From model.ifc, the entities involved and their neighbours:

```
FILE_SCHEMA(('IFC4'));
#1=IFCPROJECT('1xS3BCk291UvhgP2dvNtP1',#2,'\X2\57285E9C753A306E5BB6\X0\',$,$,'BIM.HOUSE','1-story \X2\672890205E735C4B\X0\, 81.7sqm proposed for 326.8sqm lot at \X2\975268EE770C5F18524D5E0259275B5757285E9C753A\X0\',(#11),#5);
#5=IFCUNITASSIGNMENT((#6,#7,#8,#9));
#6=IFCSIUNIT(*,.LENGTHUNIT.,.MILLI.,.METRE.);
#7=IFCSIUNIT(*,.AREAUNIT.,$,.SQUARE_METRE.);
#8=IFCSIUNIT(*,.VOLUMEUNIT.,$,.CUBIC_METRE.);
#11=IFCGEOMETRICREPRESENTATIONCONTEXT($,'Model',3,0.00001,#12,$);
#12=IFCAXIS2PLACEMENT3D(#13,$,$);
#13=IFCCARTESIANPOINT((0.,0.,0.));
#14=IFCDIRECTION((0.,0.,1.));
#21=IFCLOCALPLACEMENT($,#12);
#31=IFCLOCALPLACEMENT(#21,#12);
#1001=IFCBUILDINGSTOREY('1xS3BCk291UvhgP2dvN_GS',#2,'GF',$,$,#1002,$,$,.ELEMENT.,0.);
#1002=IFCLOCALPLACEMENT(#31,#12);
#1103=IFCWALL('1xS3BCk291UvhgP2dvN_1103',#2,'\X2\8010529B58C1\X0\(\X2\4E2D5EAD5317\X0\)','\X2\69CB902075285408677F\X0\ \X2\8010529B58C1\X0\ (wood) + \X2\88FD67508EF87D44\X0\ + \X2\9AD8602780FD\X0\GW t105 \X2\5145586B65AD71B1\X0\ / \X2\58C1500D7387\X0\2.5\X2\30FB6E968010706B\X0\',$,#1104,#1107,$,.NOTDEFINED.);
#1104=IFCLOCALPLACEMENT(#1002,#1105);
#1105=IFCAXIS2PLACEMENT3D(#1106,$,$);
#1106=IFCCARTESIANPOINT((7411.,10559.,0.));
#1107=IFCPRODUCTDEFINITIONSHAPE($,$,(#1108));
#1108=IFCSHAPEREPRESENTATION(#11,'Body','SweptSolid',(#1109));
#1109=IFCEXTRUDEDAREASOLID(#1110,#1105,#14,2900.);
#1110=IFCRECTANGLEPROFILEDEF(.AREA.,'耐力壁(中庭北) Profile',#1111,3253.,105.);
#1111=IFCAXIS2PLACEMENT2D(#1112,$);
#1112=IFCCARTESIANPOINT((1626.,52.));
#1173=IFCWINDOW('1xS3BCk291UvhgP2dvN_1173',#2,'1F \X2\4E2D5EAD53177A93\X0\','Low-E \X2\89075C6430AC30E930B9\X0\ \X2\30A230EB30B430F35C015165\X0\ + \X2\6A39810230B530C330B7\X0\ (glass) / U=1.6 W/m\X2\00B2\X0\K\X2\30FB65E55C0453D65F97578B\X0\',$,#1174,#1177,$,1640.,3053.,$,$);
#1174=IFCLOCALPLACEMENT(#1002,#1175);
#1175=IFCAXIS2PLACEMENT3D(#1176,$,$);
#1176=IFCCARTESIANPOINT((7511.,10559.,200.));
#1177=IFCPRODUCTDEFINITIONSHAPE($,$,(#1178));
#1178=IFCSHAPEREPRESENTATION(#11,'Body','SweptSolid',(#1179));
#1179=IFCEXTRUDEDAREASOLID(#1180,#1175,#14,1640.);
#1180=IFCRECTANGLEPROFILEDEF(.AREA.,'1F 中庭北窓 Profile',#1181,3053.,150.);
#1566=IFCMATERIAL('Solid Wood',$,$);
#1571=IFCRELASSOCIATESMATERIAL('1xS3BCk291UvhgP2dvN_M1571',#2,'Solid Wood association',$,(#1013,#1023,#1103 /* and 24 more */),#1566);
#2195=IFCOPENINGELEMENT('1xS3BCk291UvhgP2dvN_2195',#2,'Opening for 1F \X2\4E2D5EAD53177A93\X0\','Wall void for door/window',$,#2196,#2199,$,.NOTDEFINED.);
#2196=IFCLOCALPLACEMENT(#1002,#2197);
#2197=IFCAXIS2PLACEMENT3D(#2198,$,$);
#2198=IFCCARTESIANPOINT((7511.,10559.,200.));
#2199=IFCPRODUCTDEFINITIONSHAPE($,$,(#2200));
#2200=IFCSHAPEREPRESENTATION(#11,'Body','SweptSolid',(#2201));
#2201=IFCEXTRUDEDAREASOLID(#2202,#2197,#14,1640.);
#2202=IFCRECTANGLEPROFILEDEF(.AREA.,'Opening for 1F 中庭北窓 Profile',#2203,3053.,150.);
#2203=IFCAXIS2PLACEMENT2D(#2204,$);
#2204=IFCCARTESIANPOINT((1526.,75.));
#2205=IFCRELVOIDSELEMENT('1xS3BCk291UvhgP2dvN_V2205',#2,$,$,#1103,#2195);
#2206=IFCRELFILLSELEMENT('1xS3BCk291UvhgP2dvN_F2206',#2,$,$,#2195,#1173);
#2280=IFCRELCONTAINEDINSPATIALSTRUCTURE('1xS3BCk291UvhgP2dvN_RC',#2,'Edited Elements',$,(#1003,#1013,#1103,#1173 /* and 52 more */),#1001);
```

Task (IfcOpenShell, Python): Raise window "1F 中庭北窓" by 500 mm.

```python
import numpy as np
import ifcopenshell
import ifcopenshell.api.geometry
import ifcopenshell.util.placement
import ifcopenshell.util.unit

model = ifcopenshell.open("model.ifc")
unit_scale = ifcopenshell.util.unit.calculate_unit_scale(model)

window = model.by_guid("1xS3BCk291UvhgP2dvN_1173")
opening = window.FillsVoids[0].RelatingOpeningElement
dz = 0.5 / unit_scale

shift = np.array([0.0, 0.0, dz])
# The window is not placed relative to its opening, so move both.
for product in (opening, window):
    matrix = ifcopenshell.util.placement.get_local_placement(product.ObjectPlacement)
    matrix[:3, 3] += shift
    ifcopenshell.api.geometry.edit_object_placement(model, product=product, matrix=matrix, is_si=False)

print(f"moved by {dz * unit_scale:+.3f} m")

model.write("model_rev.ifc")
```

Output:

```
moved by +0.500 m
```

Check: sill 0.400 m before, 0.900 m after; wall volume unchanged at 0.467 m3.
